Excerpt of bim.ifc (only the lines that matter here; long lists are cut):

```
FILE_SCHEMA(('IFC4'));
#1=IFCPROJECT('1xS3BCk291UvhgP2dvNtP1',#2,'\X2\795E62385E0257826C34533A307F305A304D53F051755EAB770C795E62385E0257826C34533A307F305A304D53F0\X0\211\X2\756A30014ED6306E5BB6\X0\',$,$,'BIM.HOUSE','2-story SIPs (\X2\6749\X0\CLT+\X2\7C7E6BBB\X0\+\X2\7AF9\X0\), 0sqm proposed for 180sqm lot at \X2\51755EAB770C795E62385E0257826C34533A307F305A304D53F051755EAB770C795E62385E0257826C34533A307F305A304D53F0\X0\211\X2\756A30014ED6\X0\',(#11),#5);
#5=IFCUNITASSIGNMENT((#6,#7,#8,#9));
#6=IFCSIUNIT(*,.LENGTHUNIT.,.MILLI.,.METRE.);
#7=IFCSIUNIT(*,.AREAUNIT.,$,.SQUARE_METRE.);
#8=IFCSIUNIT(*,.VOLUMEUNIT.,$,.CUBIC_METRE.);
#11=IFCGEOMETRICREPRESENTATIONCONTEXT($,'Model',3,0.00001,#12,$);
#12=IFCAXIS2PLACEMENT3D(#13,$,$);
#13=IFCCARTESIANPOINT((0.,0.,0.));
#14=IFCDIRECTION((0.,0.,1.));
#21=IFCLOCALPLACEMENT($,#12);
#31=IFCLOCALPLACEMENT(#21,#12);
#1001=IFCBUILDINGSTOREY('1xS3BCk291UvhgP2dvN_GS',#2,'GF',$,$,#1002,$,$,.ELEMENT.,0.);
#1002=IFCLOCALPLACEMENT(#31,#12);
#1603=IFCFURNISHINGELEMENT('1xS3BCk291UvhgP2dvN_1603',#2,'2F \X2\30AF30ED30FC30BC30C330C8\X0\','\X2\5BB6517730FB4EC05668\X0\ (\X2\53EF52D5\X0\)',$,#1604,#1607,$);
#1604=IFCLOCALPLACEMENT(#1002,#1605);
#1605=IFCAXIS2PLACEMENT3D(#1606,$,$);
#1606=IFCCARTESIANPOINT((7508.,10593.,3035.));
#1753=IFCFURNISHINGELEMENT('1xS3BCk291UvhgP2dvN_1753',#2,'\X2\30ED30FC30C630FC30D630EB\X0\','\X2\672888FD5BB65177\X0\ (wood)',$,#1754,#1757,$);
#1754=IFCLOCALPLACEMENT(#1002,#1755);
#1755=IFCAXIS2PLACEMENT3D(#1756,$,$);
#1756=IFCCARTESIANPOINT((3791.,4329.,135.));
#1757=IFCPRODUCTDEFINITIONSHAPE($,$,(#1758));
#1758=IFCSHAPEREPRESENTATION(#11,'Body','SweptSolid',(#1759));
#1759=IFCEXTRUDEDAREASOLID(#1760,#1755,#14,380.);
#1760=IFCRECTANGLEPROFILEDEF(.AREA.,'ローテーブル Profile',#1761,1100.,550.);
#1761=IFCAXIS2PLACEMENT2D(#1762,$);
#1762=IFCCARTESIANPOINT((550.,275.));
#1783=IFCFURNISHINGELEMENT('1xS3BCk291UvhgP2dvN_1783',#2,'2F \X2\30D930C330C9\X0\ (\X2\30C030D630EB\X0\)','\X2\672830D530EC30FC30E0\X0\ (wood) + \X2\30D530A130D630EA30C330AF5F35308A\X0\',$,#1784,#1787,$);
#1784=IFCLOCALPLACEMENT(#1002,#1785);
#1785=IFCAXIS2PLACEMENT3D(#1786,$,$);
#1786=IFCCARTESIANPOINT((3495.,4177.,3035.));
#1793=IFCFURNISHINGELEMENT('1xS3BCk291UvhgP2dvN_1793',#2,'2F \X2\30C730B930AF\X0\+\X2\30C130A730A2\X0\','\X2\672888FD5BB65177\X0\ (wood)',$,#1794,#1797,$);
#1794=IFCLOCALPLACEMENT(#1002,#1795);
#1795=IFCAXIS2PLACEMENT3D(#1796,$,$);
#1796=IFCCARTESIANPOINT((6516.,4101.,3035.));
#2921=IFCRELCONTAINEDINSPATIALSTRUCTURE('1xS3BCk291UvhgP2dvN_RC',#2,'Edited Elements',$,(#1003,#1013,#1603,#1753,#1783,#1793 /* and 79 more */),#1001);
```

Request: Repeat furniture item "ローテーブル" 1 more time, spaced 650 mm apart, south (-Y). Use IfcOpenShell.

```python
import numpy as np
import ifcopenshell
import ifcopenshell.api.geometry
import ifcopenshell.api.root
import ifcopenshell.util.element
import ifcopenshell.util.placement

model = ifcopenshell.open("bim.ifc")


def reuse_history(source, copy):
    """copy_class also copies each property set's owner history, people and application; keep the originals."""
    for rel in copy.IsDefinedBy:
        if rel.is_a("IfcRelDefinesByProperties") and (history := rel.RelatingPropertyDefinition.OwnerHistory):
            rel.RelatingPropertyDefinition.OwnerHistory = source.OwnerHistory
            ifcopenshell.util.element.remove_deep2(model, history)


source = model.by_id(1753)
base = ifcopenshell.util.placement.get_local_placement(source.ObjectPlacement)
step = np.array([0.0, -1.0, 0.0]) * 650.0

for i in range(1, 2):
    copy = ifcopenshell.api.root.copy_class(model, product=source)
    copy.Representation = ifcopenshell.util.element.copy_deep(
        model, source.Representation, exclude=["IfcGeometricRepresentationContext", "IfcRepresentationMap"]
    )
    reuse_history(source, copy)
    matrix = base.copy()
    matrix[:3, 3] += i * step
    print("added at", matrix[:3, 3].round(3) + 0.0)
    ifcopenshell.api.geometry.edit_object_placement(model, product=copy, matrix=matrix, is_si=False)

model.write("bim_rev.ifc")
```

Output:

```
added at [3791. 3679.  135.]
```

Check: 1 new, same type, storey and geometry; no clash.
